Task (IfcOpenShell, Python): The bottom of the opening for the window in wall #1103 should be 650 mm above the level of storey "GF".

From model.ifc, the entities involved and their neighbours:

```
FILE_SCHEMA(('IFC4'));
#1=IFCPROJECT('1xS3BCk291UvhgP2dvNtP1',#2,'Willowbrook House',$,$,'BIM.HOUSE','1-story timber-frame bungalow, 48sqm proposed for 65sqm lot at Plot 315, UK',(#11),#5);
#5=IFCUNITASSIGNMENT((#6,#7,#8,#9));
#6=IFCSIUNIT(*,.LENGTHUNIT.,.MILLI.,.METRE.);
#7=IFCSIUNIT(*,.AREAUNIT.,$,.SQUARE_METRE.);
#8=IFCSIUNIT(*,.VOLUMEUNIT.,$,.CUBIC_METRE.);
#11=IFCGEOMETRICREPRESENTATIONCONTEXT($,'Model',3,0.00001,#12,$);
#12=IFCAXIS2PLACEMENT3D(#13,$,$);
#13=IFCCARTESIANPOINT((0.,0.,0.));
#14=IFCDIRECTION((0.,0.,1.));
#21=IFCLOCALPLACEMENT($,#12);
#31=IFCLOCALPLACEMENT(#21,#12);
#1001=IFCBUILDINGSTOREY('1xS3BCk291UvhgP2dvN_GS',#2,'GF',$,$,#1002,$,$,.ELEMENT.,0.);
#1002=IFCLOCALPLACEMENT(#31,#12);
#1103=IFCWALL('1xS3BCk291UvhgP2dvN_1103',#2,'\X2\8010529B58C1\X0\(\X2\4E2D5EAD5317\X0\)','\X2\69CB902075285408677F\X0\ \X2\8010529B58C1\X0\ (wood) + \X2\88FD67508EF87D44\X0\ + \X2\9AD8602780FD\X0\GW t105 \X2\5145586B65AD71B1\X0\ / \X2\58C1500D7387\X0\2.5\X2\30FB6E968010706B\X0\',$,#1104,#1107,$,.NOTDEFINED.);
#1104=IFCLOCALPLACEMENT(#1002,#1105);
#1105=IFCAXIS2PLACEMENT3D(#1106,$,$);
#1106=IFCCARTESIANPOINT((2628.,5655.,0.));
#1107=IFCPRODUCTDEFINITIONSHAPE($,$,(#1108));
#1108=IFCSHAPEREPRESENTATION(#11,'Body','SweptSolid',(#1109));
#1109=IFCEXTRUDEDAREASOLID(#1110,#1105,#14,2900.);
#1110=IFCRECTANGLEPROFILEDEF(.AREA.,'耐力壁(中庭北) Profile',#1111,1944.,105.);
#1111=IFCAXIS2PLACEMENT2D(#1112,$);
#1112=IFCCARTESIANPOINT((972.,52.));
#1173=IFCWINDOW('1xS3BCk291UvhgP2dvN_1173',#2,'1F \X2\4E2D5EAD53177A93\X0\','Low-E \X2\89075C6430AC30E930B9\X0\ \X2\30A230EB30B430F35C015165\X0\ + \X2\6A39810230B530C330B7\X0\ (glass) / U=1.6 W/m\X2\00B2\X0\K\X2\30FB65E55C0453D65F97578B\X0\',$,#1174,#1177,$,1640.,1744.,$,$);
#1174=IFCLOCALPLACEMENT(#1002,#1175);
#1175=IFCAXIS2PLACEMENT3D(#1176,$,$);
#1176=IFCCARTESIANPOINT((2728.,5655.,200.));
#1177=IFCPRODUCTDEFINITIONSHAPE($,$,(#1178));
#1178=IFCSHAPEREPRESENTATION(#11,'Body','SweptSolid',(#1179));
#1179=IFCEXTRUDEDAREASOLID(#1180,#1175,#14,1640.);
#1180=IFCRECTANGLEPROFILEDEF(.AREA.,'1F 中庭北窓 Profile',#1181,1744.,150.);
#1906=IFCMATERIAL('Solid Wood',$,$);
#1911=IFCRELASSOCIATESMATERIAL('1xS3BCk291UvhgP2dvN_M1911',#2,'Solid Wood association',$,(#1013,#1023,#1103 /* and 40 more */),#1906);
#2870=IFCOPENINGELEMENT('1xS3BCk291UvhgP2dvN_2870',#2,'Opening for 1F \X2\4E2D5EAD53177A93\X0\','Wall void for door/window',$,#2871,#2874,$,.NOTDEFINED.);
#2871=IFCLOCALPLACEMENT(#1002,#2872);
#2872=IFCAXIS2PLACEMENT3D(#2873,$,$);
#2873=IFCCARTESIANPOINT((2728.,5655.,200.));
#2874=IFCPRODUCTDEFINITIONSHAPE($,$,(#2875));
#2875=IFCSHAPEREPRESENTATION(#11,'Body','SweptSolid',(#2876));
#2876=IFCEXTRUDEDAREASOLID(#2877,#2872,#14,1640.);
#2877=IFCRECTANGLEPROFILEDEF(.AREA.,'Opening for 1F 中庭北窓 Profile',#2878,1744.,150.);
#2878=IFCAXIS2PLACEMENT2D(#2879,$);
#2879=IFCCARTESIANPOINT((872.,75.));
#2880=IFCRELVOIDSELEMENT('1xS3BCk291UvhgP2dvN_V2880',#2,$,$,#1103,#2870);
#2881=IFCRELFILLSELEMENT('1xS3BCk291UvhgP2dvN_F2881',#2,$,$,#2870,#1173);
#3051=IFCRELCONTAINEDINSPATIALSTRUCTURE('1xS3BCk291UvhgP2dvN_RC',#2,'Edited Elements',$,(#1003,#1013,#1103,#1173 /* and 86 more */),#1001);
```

```python
import numpy as np
import ifcopenshell
import ifcopenshell.api.geometry
import ifcopenshell.geom
import ifcopenshell.util.element
import ifcopenshell.util.placement
import ifcopenshell.util.shape
import ifcopenshell.util.unit

model = ifcopenshell.open("model.ifc")
unit_scale = ifcopenshell.util.unit.calculate_unit_scale(model)

window = model.by_guid("1xS3BCk291UvhgP2dvN_1173")
opening = window.FillsVoids[0].RelatingOpeningElement
storey = ifcopenshell.util.element.get_container(window, ifc_class="IfcBuildingStorey")
level = ifcopenshell.util.placement.get_local_placement(storey.ObjectPlacement)[2, 3]

# The opening's origin need not be at the sill, so measure its lowest point.
shape = ifcopenshell.geom.create_shape(ifcopenshell.geom.settings(), opening)
bottom = ifcopenshell.util.shape.get_shape_bottom_elevation(shape, shape.geometry) / unit_scale
dz = level + 0.65 / unit_scale - bottom

shift = np.array([0.0, 0.0, dz])
# The window is not placed relative to its opening, so move both.
for product in (opening, window):
    matrix = ifcopenshell.util.placement.get_local_placement(product.ObjectPlacement)
    matrix[:3, 3] += shift
    ifcopenshell.api.geometry.edit_object_placement(model, product=product, matrix=matrix, is_si=False)

print(f"moved by {dz * unit_scale:+.3f} m")

model.write("model-out.ifc")
```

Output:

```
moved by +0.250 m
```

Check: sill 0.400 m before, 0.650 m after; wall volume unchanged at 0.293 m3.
